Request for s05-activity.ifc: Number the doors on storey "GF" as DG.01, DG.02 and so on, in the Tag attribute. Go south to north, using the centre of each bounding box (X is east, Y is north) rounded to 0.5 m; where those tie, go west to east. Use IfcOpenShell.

First a look at what the model holds.

```python
import ifcopenshell
import ifcopenshell.util.element
import ifcopenshell.util.placement

model = ifcopenshell.open("s05-activity.ifc")
print(model.schema)
storey = next(s for s in model.by_type("IfcBuildingStorey") if s.Name == "GF")
doors = [e for e in ifcopenshell.util.element.get_decomposition(storey) if e.is_a("IfcDoor")]
for e in sorted(doors, key=lambda e: e.id()):
    origin = ifcopenshell.util.placement.get_local_placement(e.ObjectPlacement)[:3, 3]
    print(e.id(), e.Tag, e.Name, origin.round(2) + 0.0, sep=" | ")
```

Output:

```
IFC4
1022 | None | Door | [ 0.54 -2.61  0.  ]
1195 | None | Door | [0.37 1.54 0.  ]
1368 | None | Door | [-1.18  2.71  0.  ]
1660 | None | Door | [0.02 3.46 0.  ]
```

```python
import ifcopenshell
import ifcopenshell.geom
import ifcopenshell.util.element
import ifcopenshell.util.shape

model = ifcopenshell.open("s05-activity.ifc")
settings = ifcopenshell.geom.settings()
settings.set("use-world-coords", True)


def centre(element):
    shape = ifcopenshell.geom.create_shape(settings, element)
    return ifcopenshell.util.shape.get_bbox_centroid(shape.geometry)


storey = next(s for s in model.by_type("IfcBuildingStorey") if s.Name == "GF")
doors = [e for e in ifcopenshell.util.element.get_decomposition(storey) if e.is_a("IfcDoor")]

# Insertion points can sit at a corner or the storey origin, so sort by the geometry (in metres).
centres = {e: centre(e) for e in doors}
doors.sort(key=lambda e: (round(centres[e][1] / 0.5), centres[e][0]))

for i, e in enumerate(doors, start=1):
    number = f"DG.{i:02d}"
    e.Tag = number
    print(e.id(), number)

model.write("s05-activity_rev.ifc")
```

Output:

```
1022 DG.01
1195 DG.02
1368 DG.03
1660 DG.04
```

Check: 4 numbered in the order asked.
